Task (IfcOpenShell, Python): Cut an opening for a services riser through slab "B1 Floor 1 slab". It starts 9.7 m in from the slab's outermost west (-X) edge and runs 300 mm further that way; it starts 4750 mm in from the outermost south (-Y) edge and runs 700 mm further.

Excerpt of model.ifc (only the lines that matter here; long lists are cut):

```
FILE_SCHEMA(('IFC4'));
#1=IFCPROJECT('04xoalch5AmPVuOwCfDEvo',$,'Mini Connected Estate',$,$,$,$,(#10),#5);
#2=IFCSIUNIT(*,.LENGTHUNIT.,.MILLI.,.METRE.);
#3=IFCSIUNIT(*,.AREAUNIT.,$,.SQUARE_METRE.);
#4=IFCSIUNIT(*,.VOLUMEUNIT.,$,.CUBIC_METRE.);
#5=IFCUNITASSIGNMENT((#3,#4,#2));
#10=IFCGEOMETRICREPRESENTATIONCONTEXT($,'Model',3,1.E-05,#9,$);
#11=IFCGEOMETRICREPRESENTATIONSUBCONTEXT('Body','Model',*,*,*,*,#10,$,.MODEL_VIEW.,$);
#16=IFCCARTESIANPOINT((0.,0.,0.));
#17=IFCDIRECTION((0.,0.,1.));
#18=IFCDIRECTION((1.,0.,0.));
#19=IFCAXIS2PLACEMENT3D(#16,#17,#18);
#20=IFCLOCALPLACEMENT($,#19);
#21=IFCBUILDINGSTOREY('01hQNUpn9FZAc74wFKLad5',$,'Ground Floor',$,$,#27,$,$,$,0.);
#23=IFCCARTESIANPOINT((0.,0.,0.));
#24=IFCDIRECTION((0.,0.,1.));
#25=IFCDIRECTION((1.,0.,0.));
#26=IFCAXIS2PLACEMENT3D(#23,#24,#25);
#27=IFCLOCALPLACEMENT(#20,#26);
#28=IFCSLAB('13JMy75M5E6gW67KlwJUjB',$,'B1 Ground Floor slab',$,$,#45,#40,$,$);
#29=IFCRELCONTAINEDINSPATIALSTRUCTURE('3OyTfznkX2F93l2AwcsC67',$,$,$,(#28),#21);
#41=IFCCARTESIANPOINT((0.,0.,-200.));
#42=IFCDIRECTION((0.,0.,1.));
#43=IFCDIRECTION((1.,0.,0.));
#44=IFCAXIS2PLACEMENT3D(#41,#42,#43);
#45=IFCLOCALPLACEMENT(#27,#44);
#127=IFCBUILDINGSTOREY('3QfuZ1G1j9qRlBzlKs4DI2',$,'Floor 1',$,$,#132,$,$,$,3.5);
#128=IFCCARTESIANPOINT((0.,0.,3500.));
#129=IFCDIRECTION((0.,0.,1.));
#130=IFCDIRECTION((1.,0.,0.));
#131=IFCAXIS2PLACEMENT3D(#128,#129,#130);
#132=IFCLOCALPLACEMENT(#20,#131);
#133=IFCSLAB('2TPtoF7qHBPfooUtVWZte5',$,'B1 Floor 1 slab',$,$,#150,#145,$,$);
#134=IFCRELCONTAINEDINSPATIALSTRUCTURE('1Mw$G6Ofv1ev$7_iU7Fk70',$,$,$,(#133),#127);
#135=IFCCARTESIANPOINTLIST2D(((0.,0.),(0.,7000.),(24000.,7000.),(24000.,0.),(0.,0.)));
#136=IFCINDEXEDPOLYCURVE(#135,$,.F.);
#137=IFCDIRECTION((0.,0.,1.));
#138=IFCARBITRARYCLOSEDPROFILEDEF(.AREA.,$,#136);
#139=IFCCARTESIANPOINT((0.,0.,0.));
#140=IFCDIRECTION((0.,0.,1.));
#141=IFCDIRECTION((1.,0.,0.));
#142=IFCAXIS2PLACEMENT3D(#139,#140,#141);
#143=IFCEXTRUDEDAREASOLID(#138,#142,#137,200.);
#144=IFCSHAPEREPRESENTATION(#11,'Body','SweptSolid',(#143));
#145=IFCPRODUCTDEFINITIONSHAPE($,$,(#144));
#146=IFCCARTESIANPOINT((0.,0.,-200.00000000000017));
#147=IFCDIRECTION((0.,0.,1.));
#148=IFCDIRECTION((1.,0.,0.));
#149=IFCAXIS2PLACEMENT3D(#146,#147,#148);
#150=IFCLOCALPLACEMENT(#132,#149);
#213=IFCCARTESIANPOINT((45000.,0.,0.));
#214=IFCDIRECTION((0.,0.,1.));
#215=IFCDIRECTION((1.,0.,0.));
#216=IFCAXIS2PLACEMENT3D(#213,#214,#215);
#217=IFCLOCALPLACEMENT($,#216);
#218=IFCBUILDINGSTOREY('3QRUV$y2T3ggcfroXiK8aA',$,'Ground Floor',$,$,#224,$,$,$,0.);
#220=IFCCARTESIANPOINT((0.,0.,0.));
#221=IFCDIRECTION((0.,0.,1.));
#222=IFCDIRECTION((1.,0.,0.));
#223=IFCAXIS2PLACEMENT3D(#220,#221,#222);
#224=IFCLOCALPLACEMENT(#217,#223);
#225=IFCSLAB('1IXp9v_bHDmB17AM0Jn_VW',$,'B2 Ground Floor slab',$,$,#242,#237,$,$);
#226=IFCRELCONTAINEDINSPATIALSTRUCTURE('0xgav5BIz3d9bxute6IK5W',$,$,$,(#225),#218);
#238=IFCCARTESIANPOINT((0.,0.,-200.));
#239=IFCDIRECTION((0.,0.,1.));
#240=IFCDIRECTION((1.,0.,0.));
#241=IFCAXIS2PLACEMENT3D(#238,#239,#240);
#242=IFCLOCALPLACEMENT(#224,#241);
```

```python
import numpy as np
import ifcopenshell
import ifcopenshell.api.feature
import ifcopenshell.api.geometry
import ifcopenshell.api.root
import ifcopenshell.geom
import ifcopenshell.util.placement
import ifcopenshell.util.representation
import ifcopenshell.util.shape
import ifcopenshell.util.unit

model = ifcopenshell.open("model.ifc")
unit_scale = ifcopenshell.util.unit.calculate_unit_scale(model)
settings = ifcopenshell.geom.settings()


def volume(element):
    """Net volume in cubic metres, openings subtracted."""
    shape = ifcopenshell.geom.create_shape(settings, element)
    return ifcopenshell.util.shape.get_volume(shape.geometry)


slab = model.by_guid("2TPtoF7qHBPfooUtVWZte5")
before = volume(slab)

# Extent in the slab's own axes, in metres. The edges named are its -X and -Y sides.
slab_shape = ifcopenshell.geom.create_shape(settings, slab)
vertices = ifcopenshell.util.shape.get_vertices(slab_shape.geometry)
x_min, y_min, bottom = vertices.min(axis=0)
top = vertices[:, 2].max()

opening = ifcopenshell.api.root.create_entity(model, ifc_class="IfcOpeningElement", name="Services riser opening", predefined_type="OPENING")
context = ifcopenshell.util.representation.get_context(model, "Model", "Body", "MODEL_VIEW")
width, depth = 0.3, 0.7
outline = [(0.0, 0.0), (width, 0.0), (width, depth), (0.0, depth), (0.0, 0.0)]
# Overshoot both faces by 50 mm so the cut is clean.
shape = ifcopenshell.api.geometry.add_slab_representation(
    model, context=context, depth=top - bottom + 0.1, polyline=outline
)
ifcopenshell.api.geometry.assign_representation(model, product=opening, representation=shape)

matrix = ifcopenshell.util.placement.get_local_placement(slab.ObjectPlacement)
matrix[:, 3] = matrix @ np.append(np.array([x_min + 9.7, y_min + 4.75, bottom - 0.05]) / unit_scale, 1.0)
ifcopenshell.api.geometry.edit_object_placement(model, product=opening, matrix=matrix, is_si=False)
ifcopenshell.api.feature.add_feature(model, feature=opening, element=slab)

after = volume(slab)

print(f"slab volume {before:.3f} -> {after:.3f} m3")

model.write("model_edited.ifc")
```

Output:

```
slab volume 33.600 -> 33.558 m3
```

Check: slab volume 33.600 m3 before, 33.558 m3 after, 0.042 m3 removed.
